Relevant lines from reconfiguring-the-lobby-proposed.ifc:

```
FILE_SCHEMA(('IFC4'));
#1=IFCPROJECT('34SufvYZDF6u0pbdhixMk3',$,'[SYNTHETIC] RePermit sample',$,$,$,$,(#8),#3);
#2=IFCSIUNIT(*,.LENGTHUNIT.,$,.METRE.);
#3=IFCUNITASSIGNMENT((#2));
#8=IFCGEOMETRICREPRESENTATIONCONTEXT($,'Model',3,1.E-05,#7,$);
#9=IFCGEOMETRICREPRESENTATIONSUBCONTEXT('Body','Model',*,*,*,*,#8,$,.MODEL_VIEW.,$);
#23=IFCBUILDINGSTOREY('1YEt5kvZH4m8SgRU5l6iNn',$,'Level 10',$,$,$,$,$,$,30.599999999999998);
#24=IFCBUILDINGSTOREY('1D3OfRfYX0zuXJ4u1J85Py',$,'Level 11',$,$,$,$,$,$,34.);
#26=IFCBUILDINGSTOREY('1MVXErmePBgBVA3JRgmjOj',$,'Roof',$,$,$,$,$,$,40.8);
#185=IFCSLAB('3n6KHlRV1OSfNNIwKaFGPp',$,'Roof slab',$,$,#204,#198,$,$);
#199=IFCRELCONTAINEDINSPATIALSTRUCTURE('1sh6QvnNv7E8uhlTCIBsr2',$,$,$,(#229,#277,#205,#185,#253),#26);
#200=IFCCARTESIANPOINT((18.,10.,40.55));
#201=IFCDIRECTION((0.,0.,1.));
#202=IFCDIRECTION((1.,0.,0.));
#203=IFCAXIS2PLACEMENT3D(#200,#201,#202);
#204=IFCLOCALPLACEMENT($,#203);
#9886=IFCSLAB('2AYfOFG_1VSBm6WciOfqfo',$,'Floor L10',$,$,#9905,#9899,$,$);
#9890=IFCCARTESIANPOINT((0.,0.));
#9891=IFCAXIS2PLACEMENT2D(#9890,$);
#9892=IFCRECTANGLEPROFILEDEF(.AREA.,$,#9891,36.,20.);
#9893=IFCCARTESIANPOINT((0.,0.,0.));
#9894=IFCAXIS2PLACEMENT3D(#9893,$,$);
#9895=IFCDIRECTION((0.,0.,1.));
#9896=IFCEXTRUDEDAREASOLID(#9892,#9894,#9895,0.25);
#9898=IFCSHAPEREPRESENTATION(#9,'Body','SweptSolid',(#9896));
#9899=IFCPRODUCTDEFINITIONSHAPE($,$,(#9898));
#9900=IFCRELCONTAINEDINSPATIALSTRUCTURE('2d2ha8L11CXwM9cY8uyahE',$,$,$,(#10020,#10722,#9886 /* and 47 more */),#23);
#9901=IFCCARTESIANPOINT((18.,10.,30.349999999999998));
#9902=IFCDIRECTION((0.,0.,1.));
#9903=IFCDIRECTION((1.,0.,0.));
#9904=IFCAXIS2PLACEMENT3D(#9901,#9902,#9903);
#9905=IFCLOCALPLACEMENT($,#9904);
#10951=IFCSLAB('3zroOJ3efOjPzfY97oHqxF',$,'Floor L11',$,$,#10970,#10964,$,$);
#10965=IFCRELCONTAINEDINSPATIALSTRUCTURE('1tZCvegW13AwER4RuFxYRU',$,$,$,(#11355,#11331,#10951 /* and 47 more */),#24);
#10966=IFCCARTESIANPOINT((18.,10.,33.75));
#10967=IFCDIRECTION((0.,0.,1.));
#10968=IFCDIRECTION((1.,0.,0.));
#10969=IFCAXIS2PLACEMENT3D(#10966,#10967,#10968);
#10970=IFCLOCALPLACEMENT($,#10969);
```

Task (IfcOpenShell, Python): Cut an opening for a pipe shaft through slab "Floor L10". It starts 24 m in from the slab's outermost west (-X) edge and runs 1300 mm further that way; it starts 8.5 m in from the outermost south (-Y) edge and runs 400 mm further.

```python
import numpy as np
import ifcopenshell
import ifcopenshell.api.feature
import ifcopenshell.api.geometry
import ifcopenshell.api.root
import ifcopenshell.geom
import ifcopenshell.util.placement
import ifcopenshell.util.representation
import ifcopenshell.util.shape
import ifcopenshell.util.unit

model = ifcopenshell.open("reconfiguring-the-lobby-proposed.ifc")
unit_scale = ifcopenshell.util.unit.calculate_unit_scale(model)
settings = ifcopenshell.geom.settings()


def volume(element):
    """Net volume in cubic metres, openings subtracted."""
    shape = ifcopenshell.geom.create_shape(settings, element)
    return ifcopenshell.util.shape.get_volume(shape.geometry)


slab = model.by_id(9886)
before = volume(slab)

# Extent in the slab's own axes, in metres. The edges named are its -X and -Y sides.
slab_shape = ifcopenshell.geom.create_shape(settings, slab)
vertices = ifcopenshell.util.shape.get_vertices(slab_shape.geometry)
x_min, y_min, bottom = vertices.min(axis=0)
top = vertices[:, 2].max()

opening = ifcopenshell.api.root.create_entity(model, ifc_class="IfcOpeningElement", name="Pipe shaft opening", predefined_type="OPENING")
context = ifcopenshell.util.representation.get_context(model, "Model", "Body", "MODEL_VIEW")
width, depth = 1.3, 0.4
outline = [(0.0, 0.0), (width, 0.0), (width, depth), (0.0, depth), (0.0, 0.0)]
# Overshoot both faces by 50 mm so the cut is clean.
shape = ifcopenshell.api.geometry.add_slab_representation(
    model, context=context, depth=top - bottom + 0.1, polyline=outline
)
ifcopenshell.api.geometry.assign_representation(model, product=opening, representation=shape)

matrix = ifcopenshell.util.placement.get_local_placement(slab.ObjectPlacement)
matrix[:, 3] = matrix @ np.append(np.array([x_min + 24, y_min + 8.5, bottom - 0.05]) / unit_scale, 1.0)
ifcopenshell.api.geometry.edit_object_placement(model, product=opening, matrix=matrix, is_si=False)
ifcopenshell.api.feature.add_feature(model, feature=opening, element=slab)

after = volume(slab)

print(f"slab volume {before:.3f} -> {after:.3f} m3")

model.write("reconfiguring-the-lobby-proposed-out.ifc")
```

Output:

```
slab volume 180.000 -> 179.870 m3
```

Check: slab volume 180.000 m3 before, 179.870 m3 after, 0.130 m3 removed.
